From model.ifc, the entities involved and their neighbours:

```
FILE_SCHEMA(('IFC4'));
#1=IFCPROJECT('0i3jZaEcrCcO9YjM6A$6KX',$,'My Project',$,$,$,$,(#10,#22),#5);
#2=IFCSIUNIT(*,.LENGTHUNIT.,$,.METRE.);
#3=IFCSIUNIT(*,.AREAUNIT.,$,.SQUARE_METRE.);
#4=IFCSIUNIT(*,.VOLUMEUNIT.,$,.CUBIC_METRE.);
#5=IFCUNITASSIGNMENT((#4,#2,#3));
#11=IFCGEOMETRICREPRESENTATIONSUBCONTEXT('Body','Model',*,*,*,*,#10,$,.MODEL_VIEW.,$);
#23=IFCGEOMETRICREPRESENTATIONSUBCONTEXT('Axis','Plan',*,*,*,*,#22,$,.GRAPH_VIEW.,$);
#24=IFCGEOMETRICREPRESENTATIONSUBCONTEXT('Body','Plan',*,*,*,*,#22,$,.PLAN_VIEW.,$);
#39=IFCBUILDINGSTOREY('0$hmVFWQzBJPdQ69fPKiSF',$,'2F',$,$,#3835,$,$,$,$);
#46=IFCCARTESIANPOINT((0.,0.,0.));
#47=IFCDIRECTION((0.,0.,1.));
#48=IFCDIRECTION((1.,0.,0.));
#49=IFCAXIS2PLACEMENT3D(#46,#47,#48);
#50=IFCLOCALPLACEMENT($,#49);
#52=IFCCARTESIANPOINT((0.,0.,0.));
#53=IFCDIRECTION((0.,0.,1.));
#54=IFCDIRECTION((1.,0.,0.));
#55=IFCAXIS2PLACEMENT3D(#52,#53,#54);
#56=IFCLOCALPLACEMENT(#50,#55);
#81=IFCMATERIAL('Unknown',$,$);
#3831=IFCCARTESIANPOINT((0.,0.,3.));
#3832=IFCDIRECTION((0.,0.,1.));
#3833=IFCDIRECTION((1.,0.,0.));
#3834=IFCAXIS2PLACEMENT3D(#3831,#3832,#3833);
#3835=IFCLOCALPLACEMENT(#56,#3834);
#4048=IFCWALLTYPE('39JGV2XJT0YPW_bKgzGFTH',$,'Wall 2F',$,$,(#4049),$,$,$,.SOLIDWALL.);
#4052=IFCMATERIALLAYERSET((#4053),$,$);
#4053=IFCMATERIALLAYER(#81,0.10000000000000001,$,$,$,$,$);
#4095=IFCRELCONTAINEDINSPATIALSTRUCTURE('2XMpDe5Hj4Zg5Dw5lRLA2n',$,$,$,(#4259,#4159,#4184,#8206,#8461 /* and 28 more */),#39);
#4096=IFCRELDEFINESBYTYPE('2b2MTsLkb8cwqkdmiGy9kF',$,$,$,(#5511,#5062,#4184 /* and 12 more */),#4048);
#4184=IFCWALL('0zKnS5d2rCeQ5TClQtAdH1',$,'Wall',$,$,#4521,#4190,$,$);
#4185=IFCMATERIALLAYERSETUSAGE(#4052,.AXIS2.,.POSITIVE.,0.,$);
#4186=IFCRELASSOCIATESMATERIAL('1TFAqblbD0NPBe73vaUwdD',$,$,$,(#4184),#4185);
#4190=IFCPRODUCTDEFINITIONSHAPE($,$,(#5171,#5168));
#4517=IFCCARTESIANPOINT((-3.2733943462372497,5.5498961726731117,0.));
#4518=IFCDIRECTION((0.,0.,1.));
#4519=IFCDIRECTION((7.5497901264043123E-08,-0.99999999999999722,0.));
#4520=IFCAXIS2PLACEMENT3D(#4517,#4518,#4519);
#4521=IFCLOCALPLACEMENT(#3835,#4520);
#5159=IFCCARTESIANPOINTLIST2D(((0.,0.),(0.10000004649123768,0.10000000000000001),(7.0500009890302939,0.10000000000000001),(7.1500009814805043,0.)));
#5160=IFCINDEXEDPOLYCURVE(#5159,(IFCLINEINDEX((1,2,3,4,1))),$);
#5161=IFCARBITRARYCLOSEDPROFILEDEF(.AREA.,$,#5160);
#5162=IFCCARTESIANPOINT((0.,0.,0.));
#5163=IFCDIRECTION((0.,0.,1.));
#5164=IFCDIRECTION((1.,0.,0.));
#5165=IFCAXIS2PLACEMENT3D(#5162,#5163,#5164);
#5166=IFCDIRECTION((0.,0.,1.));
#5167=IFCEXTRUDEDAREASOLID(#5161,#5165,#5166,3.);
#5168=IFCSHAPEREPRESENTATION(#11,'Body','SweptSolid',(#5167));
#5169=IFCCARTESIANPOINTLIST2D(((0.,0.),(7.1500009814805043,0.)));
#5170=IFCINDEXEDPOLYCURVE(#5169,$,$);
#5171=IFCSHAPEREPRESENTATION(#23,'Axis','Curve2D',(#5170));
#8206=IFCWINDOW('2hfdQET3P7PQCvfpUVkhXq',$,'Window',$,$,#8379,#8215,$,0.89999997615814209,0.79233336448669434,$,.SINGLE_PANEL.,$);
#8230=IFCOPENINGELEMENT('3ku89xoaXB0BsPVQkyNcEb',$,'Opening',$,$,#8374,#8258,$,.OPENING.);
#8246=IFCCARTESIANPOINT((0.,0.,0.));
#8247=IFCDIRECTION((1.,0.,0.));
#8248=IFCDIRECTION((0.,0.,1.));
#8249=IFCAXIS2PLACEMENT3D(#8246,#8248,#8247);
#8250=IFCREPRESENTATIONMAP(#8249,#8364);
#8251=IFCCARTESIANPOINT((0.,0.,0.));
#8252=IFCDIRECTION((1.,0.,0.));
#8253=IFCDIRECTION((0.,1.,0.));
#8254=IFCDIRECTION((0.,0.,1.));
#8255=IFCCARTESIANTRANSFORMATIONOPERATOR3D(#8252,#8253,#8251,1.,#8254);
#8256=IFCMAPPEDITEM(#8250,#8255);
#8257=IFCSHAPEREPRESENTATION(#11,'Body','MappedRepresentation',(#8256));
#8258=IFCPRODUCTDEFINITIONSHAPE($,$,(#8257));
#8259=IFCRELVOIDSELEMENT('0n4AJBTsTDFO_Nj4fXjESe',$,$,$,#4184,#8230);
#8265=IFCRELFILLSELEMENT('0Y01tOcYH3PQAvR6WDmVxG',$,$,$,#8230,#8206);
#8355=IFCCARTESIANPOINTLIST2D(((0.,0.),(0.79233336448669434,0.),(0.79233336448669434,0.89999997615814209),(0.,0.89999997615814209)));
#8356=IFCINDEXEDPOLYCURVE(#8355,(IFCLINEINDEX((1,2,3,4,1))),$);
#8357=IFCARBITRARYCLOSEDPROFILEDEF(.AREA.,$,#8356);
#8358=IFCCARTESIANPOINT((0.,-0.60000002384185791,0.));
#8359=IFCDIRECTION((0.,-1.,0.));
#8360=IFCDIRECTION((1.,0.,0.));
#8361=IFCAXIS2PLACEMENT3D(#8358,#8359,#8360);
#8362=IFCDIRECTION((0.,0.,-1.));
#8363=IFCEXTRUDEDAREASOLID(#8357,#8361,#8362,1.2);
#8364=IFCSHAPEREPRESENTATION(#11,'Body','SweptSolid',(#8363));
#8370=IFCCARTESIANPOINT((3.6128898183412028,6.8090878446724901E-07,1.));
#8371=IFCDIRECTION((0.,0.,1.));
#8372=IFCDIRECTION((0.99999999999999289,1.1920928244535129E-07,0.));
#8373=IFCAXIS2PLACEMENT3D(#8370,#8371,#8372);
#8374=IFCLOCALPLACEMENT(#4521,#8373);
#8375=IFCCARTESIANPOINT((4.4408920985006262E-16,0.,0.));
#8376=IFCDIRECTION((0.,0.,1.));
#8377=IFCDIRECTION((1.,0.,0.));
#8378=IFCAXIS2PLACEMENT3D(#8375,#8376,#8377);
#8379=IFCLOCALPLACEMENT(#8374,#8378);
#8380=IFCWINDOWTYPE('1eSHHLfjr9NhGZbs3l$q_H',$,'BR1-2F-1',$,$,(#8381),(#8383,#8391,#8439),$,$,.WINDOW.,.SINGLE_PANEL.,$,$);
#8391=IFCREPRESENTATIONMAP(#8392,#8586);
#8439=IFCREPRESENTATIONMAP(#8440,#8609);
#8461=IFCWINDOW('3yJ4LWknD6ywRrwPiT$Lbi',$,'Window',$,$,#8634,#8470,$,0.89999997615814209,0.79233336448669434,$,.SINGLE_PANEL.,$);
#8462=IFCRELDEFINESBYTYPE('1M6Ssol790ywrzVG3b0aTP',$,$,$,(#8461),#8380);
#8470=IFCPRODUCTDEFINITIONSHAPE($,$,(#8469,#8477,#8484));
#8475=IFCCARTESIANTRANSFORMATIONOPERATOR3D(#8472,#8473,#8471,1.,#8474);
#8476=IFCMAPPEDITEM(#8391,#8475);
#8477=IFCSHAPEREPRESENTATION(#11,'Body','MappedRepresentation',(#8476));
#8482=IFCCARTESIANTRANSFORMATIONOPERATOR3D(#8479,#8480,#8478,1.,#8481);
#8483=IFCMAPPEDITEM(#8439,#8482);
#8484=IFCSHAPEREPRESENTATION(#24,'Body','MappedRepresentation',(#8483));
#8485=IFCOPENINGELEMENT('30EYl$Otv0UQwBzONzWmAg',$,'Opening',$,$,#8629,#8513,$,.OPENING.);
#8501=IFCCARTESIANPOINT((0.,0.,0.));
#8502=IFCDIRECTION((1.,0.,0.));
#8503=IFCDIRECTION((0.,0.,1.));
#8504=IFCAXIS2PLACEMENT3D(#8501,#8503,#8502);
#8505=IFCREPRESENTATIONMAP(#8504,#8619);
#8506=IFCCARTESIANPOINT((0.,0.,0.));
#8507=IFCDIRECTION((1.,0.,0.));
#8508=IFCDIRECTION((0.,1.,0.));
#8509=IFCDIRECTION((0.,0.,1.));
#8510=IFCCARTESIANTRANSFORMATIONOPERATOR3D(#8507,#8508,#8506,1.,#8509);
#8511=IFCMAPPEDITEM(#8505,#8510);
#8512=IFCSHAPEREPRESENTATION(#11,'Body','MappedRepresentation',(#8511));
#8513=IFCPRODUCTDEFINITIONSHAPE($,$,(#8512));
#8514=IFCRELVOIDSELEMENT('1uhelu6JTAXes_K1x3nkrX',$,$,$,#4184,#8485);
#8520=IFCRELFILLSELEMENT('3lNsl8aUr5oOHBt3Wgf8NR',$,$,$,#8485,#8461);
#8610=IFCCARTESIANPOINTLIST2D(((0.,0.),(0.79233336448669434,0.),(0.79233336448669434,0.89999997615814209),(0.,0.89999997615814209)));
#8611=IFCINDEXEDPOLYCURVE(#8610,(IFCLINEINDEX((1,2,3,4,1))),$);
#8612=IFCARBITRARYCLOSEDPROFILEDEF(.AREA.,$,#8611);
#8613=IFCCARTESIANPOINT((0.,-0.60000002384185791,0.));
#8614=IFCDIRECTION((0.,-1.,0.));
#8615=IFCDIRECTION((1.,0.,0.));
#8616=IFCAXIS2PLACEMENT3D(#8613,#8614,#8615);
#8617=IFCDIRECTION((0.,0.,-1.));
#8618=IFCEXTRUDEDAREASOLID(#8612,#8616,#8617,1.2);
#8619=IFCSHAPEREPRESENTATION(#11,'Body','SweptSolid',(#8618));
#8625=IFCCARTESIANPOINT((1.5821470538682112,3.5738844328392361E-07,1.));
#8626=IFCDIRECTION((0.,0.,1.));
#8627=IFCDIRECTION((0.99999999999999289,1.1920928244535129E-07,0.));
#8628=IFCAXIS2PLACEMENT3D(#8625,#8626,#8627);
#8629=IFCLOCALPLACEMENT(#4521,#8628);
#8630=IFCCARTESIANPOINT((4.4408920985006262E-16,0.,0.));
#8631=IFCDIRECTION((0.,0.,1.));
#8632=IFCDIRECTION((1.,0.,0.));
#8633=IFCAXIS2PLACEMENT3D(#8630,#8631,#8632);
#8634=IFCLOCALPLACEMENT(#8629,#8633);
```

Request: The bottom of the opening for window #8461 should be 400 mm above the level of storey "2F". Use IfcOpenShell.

```python
import numpy as np
import ifcopenshell
import ifcopenshell.api.geometry
import ifcopenshell.geom
import ifcopenshell.util.element
import ifcopenshell.util.placement
import ifcopenshell.util.shape
import ifcopenshell.util.unit

model = ifcopenshell.open("model.ifc")
unit_scale = ifcopenshell.util.unit.calculate_unit_scale(model)

window = model.by_guid("3yJ4LWknD6ywRrwPiT$Lbi")
opening = window.FillsVoids[0].RelatingOpeningElement
storey = ifcopenshell.util.element.get_container(window, ifc_class="IfcBuildingStorey")
level = ifcopenshell.util.placement.get_local_placement(storey.ObjectPlacement)[2, 3]

# The opening's origin need not be at the sill, so measure its lowest point.
shape = ifcopenshell.geom.create_shape(ifcopenshell.geom.settings(), opening)
bottom = ifcopenshell.util.shape.get_shape_bottom_elevation(shape, shape.geometry) / unit_scale
dz = level + 0.4 / unit_scale - bottom

shift = np.array([0.0, 0.0, dz])
# The window is placed relative to its opening, so it follows when the opening moves.
matrix = ifcopenshell.util.placement.get_local_placement(opening.ObjectPlacement)
matrix[:3, 3] += shift
ifcopenshell.api.geometry.edit_object_placement(
    model, product=opening, matrix=matrix, is_si=False, should_transform_children=True
)

print(f"moved by {dz * unit_scale:+.3f} m")

model.write("model-out.ifc")
```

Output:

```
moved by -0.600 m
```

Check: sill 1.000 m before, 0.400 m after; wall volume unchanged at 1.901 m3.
